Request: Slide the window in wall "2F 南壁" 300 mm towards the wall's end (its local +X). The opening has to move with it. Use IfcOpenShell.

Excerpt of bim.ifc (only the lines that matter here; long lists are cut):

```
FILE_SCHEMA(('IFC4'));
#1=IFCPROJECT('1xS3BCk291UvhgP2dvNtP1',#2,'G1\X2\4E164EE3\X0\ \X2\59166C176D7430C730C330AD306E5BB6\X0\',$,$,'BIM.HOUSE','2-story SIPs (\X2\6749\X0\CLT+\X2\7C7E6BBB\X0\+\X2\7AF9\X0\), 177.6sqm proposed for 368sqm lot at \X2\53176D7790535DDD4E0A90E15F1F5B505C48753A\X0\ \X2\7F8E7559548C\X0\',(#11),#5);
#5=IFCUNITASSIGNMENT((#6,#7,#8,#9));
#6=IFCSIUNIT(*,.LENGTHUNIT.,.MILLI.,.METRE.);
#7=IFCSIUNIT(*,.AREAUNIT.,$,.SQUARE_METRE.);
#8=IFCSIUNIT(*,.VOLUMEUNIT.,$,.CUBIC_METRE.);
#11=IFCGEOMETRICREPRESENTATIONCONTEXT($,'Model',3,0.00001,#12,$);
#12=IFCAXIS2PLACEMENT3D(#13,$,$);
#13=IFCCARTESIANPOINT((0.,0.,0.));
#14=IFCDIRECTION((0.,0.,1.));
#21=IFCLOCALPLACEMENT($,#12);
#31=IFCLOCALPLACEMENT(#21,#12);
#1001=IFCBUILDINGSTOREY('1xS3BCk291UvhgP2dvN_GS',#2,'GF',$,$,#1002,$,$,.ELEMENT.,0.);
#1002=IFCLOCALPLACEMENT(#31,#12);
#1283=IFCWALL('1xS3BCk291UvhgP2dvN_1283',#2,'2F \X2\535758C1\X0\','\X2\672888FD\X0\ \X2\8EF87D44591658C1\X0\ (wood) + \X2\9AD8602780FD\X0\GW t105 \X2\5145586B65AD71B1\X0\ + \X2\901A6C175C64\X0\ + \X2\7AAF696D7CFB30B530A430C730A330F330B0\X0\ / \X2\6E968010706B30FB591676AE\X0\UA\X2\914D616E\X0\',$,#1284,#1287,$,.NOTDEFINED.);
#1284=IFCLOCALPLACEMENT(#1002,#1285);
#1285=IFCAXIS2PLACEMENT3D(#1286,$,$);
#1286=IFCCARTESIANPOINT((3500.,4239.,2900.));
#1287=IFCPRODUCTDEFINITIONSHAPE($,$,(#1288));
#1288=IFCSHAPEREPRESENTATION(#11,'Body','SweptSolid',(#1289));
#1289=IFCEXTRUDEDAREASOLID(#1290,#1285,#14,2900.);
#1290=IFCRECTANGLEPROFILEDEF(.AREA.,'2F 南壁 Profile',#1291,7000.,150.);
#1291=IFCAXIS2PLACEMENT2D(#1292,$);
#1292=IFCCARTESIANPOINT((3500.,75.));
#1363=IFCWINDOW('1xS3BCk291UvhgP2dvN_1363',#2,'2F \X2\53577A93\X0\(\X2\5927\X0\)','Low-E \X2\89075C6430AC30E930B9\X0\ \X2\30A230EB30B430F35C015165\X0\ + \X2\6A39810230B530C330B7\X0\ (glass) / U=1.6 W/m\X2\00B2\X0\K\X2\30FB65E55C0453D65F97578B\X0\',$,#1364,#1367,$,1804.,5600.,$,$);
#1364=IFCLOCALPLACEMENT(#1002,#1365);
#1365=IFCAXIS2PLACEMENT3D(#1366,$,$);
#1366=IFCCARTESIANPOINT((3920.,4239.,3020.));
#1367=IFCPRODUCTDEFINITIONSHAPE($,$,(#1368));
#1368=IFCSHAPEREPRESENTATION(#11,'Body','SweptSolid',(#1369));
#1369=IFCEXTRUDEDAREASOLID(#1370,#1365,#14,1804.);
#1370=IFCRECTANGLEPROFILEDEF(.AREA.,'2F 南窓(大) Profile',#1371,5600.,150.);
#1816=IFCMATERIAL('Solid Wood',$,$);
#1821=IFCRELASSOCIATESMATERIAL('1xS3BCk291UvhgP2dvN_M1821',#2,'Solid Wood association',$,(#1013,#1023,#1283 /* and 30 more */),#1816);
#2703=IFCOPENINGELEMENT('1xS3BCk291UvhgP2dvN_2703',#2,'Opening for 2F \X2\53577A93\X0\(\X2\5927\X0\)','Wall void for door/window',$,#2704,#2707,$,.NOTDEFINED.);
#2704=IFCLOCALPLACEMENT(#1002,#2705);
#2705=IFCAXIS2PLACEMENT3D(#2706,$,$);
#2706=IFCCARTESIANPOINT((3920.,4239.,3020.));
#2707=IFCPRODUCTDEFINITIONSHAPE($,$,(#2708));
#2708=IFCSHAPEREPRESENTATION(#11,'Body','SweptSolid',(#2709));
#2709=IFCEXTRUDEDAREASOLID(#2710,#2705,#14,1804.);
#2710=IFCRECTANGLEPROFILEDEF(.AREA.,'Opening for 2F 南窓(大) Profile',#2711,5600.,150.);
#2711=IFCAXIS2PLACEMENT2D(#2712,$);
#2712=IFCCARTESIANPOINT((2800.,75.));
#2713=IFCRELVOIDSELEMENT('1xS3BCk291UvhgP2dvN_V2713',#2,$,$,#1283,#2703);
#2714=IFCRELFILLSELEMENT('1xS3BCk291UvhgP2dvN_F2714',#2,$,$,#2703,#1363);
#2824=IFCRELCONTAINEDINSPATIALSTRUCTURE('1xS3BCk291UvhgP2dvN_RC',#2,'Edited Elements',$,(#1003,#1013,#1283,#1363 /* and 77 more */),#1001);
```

```python
import ifcopenshell
import ifcopenshell.api.geometry
import ifcopenshell.util.placement
import ifcopenshell.util.unit

model = ifcopenshell.open("bim.ifc")
unit_scale = ifcopenshell.util.unit.calculate_unit_scale(model)

window = model.by_guid("1xS3BCk291UvhgP2dvN_1363")
opening = window.FillsVoids[0].RelatingOpeningElement
wall = opening.VoidsElements[0].RelatingBuildingElement

wall_matrix = ifcopenshell.util.placement.get_local_placement(wall.ObjectPlacement)
shift = wall_matrix[:3, 0] * 0.3 / unit_scale
before = ifcopenshell.util.placement.get_local_placement(window.ObjectPlacement)[:3, 3].copy()

# The window is not placed relative to its opening, so move both.
for product in (opening, window):
    matrix = ifcopenshell.util.placement.get_local_placement(product.ObjectPlacement)
    matrix[:3, 3] += shift
    ifcopenshell.api.geometry.edit_object_placement(model, product=product, matrix=matrix, is_si=False)

after = ifcopenshell.util.placement.get_local_placement(window.ObjectPlacement)[:3, 3]
print("window moved by", (after - before).round(3) + 0.0)

model.write("bim-out.ifc")
```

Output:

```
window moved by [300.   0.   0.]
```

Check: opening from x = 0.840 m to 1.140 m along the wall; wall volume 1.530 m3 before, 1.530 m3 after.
